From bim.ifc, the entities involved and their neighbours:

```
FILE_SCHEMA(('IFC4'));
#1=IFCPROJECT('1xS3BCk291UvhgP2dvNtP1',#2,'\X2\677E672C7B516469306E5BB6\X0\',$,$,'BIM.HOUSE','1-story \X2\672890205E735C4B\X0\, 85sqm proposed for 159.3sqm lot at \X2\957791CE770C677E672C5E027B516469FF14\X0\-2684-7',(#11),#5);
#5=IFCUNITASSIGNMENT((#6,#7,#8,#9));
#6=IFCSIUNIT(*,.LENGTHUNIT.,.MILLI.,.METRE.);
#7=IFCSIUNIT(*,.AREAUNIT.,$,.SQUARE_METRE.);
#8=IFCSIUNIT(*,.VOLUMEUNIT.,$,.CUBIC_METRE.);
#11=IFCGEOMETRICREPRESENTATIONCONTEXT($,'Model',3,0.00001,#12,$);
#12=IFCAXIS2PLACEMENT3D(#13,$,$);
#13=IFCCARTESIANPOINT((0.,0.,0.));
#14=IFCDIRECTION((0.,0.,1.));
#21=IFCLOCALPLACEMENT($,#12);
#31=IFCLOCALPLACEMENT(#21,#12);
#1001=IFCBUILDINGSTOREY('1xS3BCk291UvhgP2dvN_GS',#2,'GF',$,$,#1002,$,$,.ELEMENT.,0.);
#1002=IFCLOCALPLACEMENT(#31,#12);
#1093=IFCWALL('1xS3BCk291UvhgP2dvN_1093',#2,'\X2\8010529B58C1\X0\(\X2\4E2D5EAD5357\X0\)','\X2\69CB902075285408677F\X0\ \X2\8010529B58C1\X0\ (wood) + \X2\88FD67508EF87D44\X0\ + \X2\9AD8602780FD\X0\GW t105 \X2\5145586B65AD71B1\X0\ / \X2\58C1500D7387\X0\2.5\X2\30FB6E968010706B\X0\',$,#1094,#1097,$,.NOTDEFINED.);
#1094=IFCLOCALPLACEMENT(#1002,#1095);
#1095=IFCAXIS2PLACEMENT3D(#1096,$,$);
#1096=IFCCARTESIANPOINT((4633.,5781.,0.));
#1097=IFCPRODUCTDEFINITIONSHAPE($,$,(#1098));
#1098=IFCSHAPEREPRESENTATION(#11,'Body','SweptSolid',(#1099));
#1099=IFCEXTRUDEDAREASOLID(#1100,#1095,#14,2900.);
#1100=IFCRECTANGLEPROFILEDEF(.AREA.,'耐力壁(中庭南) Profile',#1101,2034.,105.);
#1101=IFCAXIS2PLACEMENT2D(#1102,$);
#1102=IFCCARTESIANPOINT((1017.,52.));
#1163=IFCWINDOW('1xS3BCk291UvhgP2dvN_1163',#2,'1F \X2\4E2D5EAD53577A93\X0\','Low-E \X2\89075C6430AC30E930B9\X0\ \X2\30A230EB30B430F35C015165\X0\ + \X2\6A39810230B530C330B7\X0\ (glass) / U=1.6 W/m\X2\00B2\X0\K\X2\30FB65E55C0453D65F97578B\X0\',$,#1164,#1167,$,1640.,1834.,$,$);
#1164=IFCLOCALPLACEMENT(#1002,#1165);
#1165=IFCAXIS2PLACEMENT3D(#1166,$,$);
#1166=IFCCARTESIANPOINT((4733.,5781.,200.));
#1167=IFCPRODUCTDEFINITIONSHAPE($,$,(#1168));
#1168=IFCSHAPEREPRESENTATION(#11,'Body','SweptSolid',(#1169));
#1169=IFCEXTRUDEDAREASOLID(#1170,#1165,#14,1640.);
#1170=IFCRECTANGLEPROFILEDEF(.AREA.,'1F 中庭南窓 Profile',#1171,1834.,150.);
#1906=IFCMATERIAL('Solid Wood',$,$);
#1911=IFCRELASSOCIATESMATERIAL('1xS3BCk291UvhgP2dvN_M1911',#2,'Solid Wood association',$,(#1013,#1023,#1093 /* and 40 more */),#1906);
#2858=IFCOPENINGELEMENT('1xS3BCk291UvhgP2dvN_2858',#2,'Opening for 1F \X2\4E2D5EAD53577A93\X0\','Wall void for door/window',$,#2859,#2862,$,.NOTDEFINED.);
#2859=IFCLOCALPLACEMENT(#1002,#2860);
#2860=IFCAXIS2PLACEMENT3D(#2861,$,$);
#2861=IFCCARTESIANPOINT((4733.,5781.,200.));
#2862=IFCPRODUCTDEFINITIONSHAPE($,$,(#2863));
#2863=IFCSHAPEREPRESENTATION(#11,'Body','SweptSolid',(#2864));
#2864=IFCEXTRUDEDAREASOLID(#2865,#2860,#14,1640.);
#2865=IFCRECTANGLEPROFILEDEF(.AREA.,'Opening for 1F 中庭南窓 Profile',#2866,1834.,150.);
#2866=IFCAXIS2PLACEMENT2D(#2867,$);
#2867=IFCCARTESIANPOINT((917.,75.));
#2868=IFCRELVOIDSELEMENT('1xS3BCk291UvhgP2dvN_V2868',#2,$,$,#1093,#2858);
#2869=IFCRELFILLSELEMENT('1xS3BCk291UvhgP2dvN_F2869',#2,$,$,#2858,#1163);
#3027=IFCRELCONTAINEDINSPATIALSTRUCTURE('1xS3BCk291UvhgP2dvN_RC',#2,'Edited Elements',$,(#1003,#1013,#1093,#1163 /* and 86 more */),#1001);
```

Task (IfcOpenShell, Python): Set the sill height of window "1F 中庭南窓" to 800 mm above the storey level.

```python
import numpy as np
import ifcopenshell
import ifcopenshell.api.geometry
import ifcopenshell.geom
import ifcopenshell.util.element
import ifcopenshell.util.placement
import ifcopenshell.util.shape
import ifcopenshell.util.unit

model = ifcopenshell.open("bim.ifc")
unit_scale = ifcopenshell.util.unit.calculate_unit_scale(model)

window = model.by_guid("1xS3BCk291UvhgP2dvN_1163")
opening = window.FillsVoids[0].RelatingOpeningElement
storey = ifcopenshell.util.element.get_container(window, ifc_class="IfcBuildingStorey")
level = ifcopenshell.util.placement.get_local_placement(storey.ObjectPlacement)[2, 3]

# The opening's origin need not be at the sill, so measure its lowest point.
shape = ifcopenshell.geom.create_shape(ifcopenshell.geom.settings(), opening)
bottom = ifcopenshell.util.shape.get_shape_bottom_elevation(shape, shape.geometry) / unit_scale
dz = level + 0.8 / unit_scale - bottom

shift = np.array([0.0, 0.0, dz])
# The window is not placed relative to its opening, so move both.
for product in (opening, window):
    matrix = ifcopenshell.util.placement.get_local_placement(product.ObjectPlacement)
    matrix[:3, 3] += shift
    ifcopenshell.api.geometry.edit_object_placement(model, product=product, matrix=matrix, is_si=False)

print(f"moved by {dz * unit_scale:+.3f} m")

model.write("bim_updated.ifc")
```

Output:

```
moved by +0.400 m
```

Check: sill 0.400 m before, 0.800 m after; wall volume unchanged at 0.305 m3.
